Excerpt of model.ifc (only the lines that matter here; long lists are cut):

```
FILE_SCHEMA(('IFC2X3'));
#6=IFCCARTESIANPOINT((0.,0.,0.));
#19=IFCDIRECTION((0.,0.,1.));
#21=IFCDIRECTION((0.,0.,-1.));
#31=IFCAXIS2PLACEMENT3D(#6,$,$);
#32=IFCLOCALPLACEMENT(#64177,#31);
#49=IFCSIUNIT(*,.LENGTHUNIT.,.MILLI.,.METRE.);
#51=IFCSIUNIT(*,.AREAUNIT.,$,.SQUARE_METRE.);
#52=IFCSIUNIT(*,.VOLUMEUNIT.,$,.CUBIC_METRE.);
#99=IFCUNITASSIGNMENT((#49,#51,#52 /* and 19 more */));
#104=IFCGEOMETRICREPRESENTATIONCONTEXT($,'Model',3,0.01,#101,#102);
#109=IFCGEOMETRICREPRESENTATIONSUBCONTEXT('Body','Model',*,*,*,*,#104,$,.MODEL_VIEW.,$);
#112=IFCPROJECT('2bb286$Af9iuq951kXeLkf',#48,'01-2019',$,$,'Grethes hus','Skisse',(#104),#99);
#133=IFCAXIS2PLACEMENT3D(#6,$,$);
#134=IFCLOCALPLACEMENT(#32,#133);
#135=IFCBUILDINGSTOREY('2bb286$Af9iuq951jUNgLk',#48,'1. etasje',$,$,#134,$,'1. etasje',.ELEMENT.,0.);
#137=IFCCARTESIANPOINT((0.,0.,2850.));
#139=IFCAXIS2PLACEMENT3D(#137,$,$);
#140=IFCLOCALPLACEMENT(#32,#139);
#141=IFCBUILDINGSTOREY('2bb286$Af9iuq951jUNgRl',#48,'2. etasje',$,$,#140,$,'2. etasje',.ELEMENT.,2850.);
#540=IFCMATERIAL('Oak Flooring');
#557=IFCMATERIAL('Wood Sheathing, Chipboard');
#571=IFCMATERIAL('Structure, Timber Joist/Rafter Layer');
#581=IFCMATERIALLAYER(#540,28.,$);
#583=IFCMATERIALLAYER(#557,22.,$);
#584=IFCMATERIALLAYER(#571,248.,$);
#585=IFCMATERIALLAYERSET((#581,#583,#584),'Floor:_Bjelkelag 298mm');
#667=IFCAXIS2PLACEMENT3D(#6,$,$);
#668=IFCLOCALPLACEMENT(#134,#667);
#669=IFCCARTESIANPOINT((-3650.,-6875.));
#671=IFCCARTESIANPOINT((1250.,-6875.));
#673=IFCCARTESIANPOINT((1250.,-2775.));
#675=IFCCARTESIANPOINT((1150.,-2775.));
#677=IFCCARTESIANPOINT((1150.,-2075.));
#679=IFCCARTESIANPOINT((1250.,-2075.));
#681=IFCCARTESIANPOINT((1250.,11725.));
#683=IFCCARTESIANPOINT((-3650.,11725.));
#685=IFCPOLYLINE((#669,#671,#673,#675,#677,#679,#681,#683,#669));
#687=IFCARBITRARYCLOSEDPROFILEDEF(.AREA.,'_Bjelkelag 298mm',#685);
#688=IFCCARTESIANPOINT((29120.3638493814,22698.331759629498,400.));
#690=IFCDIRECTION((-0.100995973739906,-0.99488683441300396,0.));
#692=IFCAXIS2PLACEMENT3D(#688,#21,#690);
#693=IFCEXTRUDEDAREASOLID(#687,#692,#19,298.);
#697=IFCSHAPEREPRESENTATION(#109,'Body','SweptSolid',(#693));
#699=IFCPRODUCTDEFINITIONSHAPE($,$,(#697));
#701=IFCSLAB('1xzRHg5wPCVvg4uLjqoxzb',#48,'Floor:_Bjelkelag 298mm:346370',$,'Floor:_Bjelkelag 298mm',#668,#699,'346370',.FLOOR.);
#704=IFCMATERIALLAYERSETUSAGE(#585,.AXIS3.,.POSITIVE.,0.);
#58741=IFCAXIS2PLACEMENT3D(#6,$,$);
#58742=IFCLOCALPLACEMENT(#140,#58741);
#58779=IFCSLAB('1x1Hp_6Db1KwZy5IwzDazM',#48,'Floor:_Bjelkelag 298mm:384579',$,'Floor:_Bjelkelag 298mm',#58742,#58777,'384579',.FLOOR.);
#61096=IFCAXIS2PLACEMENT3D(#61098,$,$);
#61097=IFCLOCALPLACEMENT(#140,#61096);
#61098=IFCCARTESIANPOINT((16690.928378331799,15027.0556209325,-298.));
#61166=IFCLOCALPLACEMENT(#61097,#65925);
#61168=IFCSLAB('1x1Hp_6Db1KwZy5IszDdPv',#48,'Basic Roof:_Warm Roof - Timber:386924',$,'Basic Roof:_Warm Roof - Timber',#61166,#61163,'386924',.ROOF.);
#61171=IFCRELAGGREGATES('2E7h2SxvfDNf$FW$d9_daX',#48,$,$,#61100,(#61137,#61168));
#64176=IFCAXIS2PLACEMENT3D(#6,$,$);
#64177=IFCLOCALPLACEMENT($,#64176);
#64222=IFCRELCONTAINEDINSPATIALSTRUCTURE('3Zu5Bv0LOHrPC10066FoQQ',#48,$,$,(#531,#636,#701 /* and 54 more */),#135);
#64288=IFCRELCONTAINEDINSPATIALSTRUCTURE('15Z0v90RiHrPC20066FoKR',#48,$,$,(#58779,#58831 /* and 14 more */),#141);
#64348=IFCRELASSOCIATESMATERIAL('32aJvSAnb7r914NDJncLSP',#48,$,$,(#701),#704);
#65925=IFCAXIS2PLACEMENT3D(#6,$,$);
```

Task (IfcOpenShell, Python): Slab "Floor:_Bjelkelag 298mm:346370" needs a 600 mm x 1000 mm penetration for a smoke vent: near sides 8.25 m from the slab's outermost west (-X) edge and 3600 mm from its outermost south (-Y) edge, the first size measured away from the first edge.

```python
import numpy as np
import ifcopenshell
import ifcopenshell.api.feature
import ifcopenshell.api.geometry
import ifcopenshell.api.root
import ifcopenshell.geom
import ifcopenshell.util.placement
import ifcopenshell.util.representation
import ifcopenshell.util.shape
import ifcopenshell.util.unit

model = ifcopenshell.open("model.ifc")
unit_scale = ifcopenshell.util.unit.calculate_unit_scale(model)
settings = ifcopenshell.geom.settings()


def volume(element):
    """Net volume in cubic metres, openings subtracted."""
    shape = ifcopenshell.geom.create_shape(settings, element)
    return ifcopenshell.util.shape.get_volume(shape.geometry)


slab = model.by_guid("1xzRHg5wPCVvg4uLjqoxzb")
before = volume(slab)

# Extent in the slab's own axes, in metres. The edges named are its -X and -Y sides.
slab_shape = ifcopenshell.geom.create_shape(settings, slab)
vertices = ifcopenshell.util.shape.get_vertices(slab_shape.geometry)
x_min, y_min, bottom = vertices.min(axis=0)
top = vertices[:, 2].max()

opening = ifcopenshell.api.root.create_entity(model, ifc_class="IfcOpeningElement", name="Smoke vent opening")
context = ifcopenshell.util.representation.get_context(model, "Model", "Body", "MODEL_VIEW")
width, depth = 0.6, 1
outline = [(0.0, 0.0), (width, 0.0), (width, depth), (0.0, depth), (0.0, 0.0)]
# Overshoot both faces by 50 mm so the cut is clean.
shape = ifcopenshell.api.geometry.add_slab_representation(
    model, context=context, depth=top - bottom + 0.1, polyline=outline
)
ifcopenshell.api.geometry.assign_representation(model, product=opening, representation=shape)

matrix = ifcopenshell.util.placement.get_local_placement(slab.ObjectPlacement)
matrix[:, 3] = matrix @ np.append(np.array([x_min + 8.25, y_min + 3.6, bottom - 0.05]) / unit_scale, 1.0)
ifcopenshell.api.geometry.edit_object_placement(model, product=opening, matrix=matrix, is_si=False)
ifcopenshell.api.feature.add_feature(model, feature=opening, element=slab)

after = volume(slab)

print(f"slab volume {before:.3f} -> {after:.3f} m3")

model.write("model_v2.ifc")
```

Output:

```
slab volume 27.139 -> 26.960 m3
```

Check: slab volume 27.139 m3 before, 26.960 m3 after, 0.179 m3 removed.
